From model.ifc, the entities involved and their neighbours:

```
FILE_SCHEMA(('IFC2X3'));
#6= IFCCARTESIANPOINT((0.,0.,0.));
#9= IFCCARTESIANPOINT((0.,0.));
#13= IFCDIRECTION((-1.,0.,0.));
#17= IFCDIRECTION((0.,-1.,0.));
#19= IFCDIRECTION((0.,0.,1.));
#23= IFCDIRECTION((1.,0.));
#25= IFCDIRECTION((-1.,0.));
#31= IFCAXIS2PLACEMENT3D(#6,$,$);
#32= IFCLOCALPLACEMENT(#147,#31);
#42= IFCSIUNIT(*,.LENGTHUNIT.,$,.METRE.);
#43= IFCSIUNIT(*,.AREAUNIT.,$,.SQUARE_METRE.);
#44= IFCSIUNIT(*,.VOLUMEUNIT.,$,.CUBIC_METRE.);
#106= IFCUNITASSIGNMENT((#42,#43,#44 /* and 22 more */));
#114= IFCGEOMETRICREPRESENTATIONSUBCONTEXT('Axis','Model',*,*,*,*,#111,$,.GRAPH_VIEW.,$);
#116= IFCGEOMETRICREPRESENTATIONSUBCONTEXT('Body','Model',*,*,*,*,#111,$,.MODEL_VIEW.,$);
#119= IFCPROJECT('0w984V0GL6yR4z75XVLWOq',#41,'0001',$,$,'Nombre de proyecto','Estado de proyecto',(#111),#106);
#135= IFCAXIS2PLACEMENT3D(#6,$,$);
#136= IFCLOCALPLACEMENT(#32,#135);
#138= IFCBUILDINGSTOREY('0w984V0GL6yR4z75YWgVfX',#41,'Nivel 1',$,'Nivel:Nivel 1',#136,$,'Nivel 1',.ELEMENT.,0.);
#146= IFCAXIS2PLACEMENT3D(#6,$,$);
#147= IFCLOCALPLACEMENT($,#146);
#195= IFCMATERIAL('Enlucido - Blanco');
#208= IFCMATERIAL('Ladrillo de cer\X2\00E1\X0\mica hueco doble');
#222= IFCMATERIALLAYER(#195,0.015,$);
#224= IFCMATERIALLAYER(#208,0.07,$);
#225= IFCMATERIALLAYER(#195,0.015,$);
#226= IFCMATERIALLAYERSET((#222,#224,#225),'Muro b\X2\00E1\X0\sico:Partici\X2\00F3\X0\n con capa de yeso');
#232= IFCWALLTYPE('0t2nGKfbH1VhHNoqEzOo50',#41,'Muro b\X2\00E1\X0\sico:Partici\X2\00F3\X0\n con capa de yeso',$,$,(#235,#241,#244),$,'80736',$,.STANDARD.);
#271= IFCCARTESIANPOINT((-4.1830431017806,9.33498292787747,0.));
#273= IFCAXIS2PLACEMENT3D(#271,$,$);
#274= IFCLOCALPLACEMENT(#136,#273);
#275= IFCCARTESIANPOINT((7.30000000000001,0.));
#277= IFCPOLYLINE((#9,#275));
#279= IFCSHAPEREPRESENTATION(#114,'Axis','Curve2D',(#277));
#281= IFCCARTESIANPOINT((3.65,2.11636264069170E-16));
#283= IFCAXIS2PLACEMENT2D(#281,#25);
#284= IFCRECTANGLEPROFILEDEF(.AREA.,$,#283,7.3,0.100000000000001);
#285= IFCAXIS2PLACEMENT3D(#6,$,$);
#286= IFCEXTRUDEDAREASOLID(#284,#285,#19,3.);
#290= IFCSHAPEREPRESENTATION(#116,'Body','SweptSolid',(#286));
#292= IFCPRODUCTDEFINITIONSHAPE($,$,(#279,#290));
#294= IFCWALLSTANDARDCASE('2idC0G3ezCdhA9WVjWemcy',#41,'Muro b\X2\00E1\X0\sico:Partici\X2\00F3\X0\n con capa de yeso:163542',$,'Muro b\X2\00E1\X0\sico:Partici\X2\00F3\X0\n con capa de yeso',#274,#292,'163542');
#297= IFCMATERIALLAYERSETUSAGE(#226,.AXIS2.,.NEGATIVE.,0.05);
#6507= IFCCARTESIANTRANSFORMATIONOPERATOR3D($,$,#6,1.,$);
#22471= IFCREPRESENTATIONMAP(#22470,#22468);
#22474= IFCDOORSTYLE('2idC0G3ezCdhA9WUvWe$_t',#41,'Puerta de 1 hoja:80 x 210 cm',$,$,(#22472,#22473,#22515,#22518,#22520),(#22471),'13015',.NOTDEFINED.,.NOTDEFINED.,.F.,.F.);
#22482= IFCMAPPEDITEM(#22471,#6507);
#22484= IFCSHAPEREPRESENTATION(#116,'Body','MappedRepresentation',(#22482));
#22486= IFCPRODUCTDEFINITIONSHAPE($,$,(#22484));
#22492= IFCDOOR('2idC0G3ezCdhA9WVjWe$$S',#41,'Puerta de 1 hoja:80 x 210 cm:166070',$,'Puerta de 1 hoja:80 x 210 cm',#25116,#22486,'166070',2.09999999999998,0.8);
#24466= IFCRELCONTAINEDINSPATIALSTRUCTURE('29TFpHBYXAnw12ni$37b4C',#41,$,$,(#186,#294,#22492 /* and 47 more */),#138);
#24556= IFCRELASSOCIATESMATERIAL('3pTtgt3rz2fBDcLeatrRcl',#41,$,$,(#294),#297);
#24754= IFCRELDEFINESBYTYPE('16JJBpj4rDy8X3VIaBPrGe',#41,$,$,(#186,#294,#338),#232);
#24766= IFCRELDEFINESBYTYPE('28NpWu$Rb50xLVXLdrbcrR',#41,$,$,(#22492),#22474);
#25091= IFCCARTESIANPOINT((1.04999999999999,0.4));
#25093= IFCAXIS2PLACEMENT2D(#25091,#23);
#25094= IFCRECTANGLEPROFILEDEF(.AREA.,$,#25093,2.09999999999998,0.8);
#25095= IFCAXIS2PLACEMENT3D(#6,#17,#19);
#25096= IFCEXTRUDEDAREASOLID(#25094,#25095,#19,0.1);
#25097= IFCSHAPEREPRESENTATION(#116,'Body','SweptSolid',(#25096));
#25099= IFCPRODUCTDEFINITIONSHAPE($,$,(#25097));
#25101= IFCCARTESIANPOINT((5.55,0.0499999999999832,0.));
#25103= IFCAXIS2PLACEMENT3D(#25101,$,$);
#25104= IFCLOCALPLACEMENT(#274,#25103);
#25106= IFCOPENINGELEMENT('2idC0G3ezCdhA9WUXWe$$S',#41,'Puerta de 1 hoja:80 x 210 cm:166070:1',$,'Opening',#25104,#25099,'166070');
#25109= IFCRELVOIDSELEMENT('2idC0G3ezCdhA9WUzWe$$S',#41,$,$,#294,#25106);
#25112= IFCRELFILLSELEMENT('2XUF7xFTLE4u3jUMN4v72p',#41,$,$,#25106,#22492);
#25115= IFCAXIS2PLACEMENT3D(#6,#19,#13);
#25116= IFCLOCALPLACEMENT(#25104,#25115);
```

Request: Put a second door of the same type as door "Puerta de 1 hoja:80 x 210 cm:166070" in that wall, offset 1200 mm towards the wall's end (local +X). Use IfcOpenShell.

```python
import ifcopenshell
import ifcopenshell.api.feature
import ifcopenshell.api.geometry
import ifcopenshell.api.root
import ifcopenshell.geom
import ifcopenshell.util.element
import ifcopenshell.util.placement
import ifcopenshell.util.shape
import ifcopenshell.util.unit

model = ifcopenshell.open("model.ifc")
unit_scale = ifcopenshell.util.unit.calculate_unit_scale(model)
settings = ifcopenshell.geom.settings()


def volume(element):
    """Net volume in cubic metres, openings subtracted."""
    shape = ifcopenshell.geom.create_shape(settings, element)
    return ifcopenshell.util.shape.get_volume(shape.geometry)


def reuse_history(source, copy):
    """copy_class also copies each property set's owner history, people and application; keep the originals."""
    for rel in copy.IsDefinedBy:
        if rel.is_a("IfcRelDefinesByProperties") and (history := rel.RelatingPropertyDefinition.OwnerHistory):
            rel.RelatingPropertyDefinition.OwnerHistory = source.OwnerHistory
            ifcopenshell.util.element.remove_deep2(model, history)


door = model.by_guid("2idC0G3ezCdhA9WVjWe$$S")
opening = door.FillsVoids[0].RelatingOpeningElement
wall = opening.VoidsElements[0].RelatingBuildingElement
before = volume(wall)
shift = ifcopenshell.util.placement.get_local_placement(wall.ObjectPlacement)[:3, 0] * 1.2 / unit_scale

# copy_class copies the void relationship, type, container and properties, but no geometry.
new_opening = ifcopenshell.api.root.copy_class(model, product=opening)
new_opening.Representation = ifcopenshell.util.element.copy_deep(
    model, opening.Representation, exclude=["IfcGeometricRepresentationContext", "IfcRepresentationMap"]
)
new_opening.Name = "Puerta de 1 hoja:80 x 210 cm"
new_opening.Tag = None
new_door = ifcopenshell.api.root.copy_class(model, product=door)
new_door.Representation = ifcopenshell.util.element.copy_deep(
    model, door.Representation, exclude=["IfcGeometricRepresentationContext", "IfcRepresentationMap"]
)
new_door.Name = "Puerta de 1 hoja:80 x 210 cm"
new_door.Tag = None
reuse_history(door, new_door)
fills = ifcopenshell.api.feature.add_filling(model, opening=new_opening, element=new_door)
fills.OwnerHistory = new_door.OwnerHistory  # required in IFC2X3

for old, new in ((opening, new_opening), (door, new_door)):
    matrix = ifcopenshell.util.placement.get_local_placement(old.ObjectPlacement)
    matrix[:3, 3] += shift
    ifcopenshell.api.geometry.edit_object_placement(model, product=new, matrix=matrix, is_si=False)

after = volume(wall)

print(f"wall volume {before:.3f} -> {after:.3f} m3")

model.write("model_v2.ifc")
```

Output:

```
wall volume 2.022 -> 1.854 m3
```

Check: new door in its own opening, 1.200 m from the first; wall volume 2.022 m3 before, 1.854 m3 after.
